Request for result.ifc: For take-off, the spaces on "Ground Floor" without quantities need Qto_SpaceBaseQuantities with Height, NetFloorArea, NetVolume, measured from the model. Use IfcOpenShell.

First a look at what the model holds.

```python
import ifcopenshell
import ifcopenshell.util.element
import ifcopenshell.util.unit

model = ifcopenshell.open("result.ifc")
print(model.schema)
for unit_type in ("LENGTHUNIT", "AREAUNIT", "VOLUMEUNIT"):
    print(unit_type, ifcopenshell.util.unit.calculate_unit_scale(model, unit_type))
storey = next(s for s in model.by_type("IfcBuildingStorey") if s.Name == "Ground Floor")
spaces = [e for e in ifcopenshell.util.element.get_decomposition(storey) if e.is_a("IfcSpace")]
for e in sorted(spaces, key=lambda e: e.id()):
    print(e.id(), e.is_a(), e.Name, list(ifcopenshell.util.element.get_psets(e, qtos_only=True)), sep=" | ")
```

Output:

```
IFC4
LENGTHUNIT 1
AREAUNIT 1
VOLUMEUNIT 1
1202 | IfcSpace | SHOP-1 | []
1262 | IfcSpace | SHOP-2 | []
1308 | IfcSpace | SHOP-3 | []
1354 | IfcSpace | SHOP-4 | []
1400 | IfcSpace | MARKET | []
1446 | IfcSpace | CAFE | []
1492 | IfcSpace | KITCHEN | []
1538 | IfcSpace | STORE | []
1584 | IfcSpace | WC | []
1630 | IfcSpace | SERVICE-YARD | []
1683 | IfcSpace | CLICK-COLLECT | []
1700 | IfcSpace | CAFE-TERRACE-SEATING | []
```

```python
import ifcopenshell
import ifcopenshell.api.pset
import ifcopenshell.geom
import ifcopenshell.util.element
import ifcopenshell.util.shape
import ifcopenshell.util.unit

model = ifcopenshell.open("result.ifc")
unit_scale = ifcopenshell.util.unit.calculate_unit_scale(model)
area_scale = ifcopenshell.util.unit.calculate_unit_scale(model, "AREAUNIT")
volume_scale = ifcopenshell.util.unit.calculate_unit_scale(model, "VOLUMEUNIT")
settings = ifcopenshell.geom.settings()

storey = next(s for s in model.by_type("IfcBuildingStorey") if s.Name == "Ground Floor")
spaces = [e for e in ifcopenshell.util.element.get_decomposition(storey) if e.is_a("IfcSpace")]

for e in sorted(spaces, key=lambda e: e.id()):
    if ifcopenshell.util.element.get_psets(e, qtos_only=True, should_inherit=False):
        continue
    # Geometry comes back in metres, in the element's own axes.
    shape = ifcopenshell.geom.create_shape(settings, e)
    values = {
        "Height": ifcopenshell.util.shape.get_z(shape.geometry) / unit_scale,
        "NetFloorArea": ifcopenshell.util.shape.get_footprint_area(shape.geometry) / area_scale,
        "NetVolume": ifcopenshell.util.shape.get_volume(shape.geometry) / volume_scale,
    }
    qto = ifcopenshell.api.pset.add_qto(model, product=e, name="Qto_SpaceBaseQuantities")
    ifcopenshell.api.pset.edit_qto(model, qto=qto, properties=values)
    print(e.id(), {k: round(v, 3) for k, v in values.items()})

model.write("result_updated.ifc")
```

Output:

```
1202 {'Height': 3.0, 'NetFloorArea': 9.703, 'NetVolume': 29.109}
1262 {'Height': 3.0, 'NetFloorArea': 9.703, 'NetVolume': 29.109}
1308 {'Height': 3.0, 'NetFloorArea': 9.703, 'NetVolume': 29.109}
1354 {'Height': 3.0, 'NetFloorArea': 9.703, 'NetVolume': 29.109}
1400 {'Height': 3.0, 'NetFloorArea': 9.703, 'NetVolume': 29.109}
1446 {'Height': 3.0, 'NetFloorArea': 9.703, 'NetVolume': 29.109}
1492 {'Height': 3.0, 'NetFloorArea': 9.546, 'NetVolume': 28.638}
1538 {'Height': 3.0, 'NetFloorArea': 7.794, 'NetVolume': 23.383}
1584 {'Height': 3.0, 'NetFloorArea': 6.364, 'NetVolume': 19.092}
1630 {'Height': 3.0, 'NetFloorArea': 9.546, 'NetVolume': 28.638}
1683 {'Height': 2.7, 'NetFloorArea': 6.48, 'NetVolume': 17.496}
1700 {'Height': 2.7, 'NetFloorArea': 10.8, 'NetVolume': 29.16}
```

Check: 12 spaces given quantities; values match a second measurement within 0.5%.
